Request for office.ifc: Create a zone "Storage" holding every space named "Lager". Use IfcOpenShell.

First a look at what the model holds.

```python
import ifcopenshell

model = ifcopenshell.open("office.ifc")
print(model.schema)
seen = {}
for space in model.by_type("IfcSpace"):
    seen[space.LongName] = seen.get(space.LongName, 0) + 1
for name, count in sorted(seen.items(), key=str):
    print(count, "x", name)
print("zones:", [z.Name for z in model.by_type("IfcZone")][:20])
```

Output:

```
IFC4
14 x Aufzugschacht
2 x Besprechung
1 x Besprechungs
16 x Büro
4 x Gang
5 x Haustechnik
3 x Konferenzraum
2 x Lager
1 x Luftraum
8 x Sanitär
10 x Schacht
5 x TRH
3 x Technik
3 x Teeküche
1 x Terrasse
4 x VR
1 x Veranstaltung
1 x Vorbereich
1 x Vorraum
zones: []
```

```python
import ifcopenshell
import ifcopenshell.api.group
import ifcopenshell.api.root

model = ifcopenshell.open("office.ifc")

names = {"Lager"}
spaces = [s for s in model.by_type("IfcSpace") if s.LongName in names]

zone = ifcopenshell.api.root.create_entity(model, ifc_class="IfcZone", name="Storage")
ifcopenshell.api.group.assign_group(model, products=spaces, group=zone)
print(len(spaces), "spaces in", zone.Name)

model.write("office_rev.ifc")
```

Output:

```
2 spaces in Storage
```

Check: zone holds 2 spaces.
